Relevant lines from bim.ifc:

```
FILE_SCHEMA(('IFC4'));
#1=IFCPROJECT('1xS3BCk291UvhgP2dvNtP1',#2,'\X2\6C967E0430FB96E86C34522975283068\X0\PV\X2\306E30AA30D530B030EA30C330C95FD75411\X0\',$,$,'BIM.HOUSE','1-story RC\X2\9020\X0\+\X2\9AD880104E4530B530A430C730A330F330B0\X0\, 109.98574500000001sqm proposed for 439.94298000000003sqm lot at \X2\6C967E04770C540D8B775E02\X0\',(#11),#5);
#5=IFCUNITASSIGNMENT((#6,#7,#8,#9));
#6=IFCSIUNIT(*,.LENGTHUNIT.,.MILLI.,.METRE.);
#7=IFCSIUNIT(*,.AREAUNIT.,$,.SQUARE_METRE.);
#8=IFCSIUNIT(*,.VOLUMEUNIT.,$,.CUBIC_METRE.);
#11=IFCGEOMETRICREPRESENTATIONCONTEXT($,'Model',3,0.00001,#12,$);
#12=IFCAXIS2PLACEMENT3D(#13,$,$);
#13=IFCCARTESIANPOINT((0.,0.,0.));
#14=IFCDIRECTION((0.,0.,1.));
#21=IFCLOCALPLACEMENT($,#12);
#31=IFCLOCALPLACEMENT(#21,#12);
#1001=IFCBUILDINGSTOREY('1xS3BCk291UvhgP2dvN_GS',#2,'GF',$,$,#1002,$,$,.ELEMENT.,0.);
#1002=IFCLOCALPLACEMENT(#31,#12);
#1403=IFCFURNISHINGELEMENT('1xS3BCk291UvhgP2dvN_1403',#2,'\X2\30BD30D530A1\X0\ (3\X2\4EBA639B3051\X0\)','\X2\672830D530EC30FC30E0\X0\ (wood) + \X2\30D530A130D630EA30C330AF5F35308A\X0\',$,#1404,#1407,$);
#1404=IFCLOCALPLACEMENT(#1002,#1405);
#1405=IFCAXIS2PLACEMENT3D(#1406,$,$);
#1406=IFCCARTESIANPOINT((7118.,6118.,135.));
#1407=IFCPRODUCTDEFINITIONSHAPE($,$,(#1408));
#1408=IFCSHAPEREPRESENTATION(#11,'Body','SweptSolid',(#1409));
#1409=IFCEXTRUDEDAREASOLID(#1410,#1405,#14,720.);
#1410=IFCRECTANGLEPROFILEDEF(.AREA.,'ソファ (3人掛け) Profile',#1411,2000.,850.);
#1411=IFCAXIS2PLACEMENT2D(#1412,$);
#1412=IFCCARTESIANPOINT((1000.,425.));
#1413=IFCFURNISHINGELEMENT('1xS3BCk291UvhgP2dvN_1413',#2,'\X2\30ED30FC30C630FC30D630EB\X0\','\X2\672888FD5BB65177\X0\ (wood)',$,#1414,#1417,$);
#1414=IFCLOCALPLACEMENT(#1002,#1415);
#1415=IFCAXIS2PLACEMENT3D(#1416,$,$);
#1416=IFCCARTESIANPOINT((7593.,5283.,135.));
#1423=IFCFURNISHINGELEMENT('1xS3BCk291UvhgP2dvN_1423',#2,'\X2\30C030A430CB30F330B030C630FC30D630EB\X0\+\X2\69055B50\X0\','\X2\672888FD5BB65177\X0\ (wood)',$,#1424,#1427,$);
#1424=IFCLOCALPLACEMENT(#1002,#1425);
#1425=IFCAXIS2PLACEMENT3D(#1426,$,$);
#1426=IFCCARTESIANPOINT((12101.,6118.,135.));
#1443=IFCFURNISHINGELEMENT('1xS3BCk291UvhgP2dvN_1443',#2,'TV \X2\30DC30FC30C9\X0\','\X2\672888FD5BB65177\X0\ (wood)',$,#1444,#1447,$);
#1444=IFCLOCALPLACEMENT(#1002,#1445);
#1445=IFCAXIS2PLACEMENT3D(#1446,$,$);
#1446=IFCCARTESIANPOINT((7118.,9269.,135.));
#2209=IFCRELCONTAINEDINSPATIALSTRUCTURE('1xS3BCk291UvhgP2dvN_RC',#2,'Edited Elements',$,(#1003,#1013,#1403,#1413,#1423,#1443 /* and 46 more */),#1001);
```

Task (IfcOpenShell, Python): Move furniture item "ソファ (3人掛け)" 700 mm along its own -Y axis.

```python
import ifcopenshell
import ifcopenshell.api.geometry
import ifcopenshell.util.placement

model = ifcopenshell.open("bim.ifc")

item = model.by_id(1403)
matrix = ifcopenshell.util.placement.get_local_placement(item.ObjectPlacement)
matrix[:3, 3] -= matrix[:3, 1] * 700.0
ifcopenshell.api.geometry.edit_object_placement(model, product=item, matrix=matrix, is_si=False)

print(ifcopenshell.util.placement.get_local_placement(item.ObjectPlacement).round(3) + 0.0)

model.write("bim-out.ifc")
```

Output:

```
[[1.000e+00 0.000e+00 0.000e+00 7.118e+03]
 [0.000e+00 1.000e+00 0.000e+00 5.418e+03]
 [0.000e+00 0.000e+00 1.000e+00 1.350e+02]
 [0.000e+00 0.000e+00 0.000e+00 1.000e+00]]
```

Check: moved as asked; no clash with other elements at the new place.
